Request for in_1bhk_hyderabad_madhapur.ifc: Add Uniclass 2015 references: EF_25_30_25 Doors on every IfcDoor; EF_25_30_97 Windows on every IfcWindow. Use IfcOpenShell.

First a look at what the model holds.

```python
import ifcopenshell

model = ifcopenshell.open("in_1bhk_hyderabad_madhapur.ifc")
print(model.schema)
print("classifications:", [c.Name for c in model.by_type("IfcClassification")])
for ifc_class in ("IfcDoor", "IfcRoof", "IfcStair", "IfcWall", "IfcWindow"):
    print(ifc_class, len(model.by_type(ifc_class)))
```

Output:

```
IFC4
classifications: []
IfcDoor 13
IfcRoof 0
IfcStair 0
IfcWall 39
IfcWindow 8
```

```python
import ifcopenshell
import ifcopenshell.api.classification

model = ifcopenshell.open("in_1bhk_hyderabad_madhapur.ifc")

system = ifcopenshell.api.classification.add_classification(model, classification="Uniclass 2015")

codes = {
    "IfcDoor": ("EF_25_30_25", "Doors"),
    "IfcWindow": ("EF_25_30_97", "Windows"),
}
for ifc_class, (code, name) in codes.items():
    products = model.by_type(ifc_class)
    ifcopenshell.api.classification.add_reference(
        model, products=products, classification=system, identification=code, name=name
    )
    print(code, len(products))

model.write("in_1bhk_hyderabad_madhapur_edited.ifc")
```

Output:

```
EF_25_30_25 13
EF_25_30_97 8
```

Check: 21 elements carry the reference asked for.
